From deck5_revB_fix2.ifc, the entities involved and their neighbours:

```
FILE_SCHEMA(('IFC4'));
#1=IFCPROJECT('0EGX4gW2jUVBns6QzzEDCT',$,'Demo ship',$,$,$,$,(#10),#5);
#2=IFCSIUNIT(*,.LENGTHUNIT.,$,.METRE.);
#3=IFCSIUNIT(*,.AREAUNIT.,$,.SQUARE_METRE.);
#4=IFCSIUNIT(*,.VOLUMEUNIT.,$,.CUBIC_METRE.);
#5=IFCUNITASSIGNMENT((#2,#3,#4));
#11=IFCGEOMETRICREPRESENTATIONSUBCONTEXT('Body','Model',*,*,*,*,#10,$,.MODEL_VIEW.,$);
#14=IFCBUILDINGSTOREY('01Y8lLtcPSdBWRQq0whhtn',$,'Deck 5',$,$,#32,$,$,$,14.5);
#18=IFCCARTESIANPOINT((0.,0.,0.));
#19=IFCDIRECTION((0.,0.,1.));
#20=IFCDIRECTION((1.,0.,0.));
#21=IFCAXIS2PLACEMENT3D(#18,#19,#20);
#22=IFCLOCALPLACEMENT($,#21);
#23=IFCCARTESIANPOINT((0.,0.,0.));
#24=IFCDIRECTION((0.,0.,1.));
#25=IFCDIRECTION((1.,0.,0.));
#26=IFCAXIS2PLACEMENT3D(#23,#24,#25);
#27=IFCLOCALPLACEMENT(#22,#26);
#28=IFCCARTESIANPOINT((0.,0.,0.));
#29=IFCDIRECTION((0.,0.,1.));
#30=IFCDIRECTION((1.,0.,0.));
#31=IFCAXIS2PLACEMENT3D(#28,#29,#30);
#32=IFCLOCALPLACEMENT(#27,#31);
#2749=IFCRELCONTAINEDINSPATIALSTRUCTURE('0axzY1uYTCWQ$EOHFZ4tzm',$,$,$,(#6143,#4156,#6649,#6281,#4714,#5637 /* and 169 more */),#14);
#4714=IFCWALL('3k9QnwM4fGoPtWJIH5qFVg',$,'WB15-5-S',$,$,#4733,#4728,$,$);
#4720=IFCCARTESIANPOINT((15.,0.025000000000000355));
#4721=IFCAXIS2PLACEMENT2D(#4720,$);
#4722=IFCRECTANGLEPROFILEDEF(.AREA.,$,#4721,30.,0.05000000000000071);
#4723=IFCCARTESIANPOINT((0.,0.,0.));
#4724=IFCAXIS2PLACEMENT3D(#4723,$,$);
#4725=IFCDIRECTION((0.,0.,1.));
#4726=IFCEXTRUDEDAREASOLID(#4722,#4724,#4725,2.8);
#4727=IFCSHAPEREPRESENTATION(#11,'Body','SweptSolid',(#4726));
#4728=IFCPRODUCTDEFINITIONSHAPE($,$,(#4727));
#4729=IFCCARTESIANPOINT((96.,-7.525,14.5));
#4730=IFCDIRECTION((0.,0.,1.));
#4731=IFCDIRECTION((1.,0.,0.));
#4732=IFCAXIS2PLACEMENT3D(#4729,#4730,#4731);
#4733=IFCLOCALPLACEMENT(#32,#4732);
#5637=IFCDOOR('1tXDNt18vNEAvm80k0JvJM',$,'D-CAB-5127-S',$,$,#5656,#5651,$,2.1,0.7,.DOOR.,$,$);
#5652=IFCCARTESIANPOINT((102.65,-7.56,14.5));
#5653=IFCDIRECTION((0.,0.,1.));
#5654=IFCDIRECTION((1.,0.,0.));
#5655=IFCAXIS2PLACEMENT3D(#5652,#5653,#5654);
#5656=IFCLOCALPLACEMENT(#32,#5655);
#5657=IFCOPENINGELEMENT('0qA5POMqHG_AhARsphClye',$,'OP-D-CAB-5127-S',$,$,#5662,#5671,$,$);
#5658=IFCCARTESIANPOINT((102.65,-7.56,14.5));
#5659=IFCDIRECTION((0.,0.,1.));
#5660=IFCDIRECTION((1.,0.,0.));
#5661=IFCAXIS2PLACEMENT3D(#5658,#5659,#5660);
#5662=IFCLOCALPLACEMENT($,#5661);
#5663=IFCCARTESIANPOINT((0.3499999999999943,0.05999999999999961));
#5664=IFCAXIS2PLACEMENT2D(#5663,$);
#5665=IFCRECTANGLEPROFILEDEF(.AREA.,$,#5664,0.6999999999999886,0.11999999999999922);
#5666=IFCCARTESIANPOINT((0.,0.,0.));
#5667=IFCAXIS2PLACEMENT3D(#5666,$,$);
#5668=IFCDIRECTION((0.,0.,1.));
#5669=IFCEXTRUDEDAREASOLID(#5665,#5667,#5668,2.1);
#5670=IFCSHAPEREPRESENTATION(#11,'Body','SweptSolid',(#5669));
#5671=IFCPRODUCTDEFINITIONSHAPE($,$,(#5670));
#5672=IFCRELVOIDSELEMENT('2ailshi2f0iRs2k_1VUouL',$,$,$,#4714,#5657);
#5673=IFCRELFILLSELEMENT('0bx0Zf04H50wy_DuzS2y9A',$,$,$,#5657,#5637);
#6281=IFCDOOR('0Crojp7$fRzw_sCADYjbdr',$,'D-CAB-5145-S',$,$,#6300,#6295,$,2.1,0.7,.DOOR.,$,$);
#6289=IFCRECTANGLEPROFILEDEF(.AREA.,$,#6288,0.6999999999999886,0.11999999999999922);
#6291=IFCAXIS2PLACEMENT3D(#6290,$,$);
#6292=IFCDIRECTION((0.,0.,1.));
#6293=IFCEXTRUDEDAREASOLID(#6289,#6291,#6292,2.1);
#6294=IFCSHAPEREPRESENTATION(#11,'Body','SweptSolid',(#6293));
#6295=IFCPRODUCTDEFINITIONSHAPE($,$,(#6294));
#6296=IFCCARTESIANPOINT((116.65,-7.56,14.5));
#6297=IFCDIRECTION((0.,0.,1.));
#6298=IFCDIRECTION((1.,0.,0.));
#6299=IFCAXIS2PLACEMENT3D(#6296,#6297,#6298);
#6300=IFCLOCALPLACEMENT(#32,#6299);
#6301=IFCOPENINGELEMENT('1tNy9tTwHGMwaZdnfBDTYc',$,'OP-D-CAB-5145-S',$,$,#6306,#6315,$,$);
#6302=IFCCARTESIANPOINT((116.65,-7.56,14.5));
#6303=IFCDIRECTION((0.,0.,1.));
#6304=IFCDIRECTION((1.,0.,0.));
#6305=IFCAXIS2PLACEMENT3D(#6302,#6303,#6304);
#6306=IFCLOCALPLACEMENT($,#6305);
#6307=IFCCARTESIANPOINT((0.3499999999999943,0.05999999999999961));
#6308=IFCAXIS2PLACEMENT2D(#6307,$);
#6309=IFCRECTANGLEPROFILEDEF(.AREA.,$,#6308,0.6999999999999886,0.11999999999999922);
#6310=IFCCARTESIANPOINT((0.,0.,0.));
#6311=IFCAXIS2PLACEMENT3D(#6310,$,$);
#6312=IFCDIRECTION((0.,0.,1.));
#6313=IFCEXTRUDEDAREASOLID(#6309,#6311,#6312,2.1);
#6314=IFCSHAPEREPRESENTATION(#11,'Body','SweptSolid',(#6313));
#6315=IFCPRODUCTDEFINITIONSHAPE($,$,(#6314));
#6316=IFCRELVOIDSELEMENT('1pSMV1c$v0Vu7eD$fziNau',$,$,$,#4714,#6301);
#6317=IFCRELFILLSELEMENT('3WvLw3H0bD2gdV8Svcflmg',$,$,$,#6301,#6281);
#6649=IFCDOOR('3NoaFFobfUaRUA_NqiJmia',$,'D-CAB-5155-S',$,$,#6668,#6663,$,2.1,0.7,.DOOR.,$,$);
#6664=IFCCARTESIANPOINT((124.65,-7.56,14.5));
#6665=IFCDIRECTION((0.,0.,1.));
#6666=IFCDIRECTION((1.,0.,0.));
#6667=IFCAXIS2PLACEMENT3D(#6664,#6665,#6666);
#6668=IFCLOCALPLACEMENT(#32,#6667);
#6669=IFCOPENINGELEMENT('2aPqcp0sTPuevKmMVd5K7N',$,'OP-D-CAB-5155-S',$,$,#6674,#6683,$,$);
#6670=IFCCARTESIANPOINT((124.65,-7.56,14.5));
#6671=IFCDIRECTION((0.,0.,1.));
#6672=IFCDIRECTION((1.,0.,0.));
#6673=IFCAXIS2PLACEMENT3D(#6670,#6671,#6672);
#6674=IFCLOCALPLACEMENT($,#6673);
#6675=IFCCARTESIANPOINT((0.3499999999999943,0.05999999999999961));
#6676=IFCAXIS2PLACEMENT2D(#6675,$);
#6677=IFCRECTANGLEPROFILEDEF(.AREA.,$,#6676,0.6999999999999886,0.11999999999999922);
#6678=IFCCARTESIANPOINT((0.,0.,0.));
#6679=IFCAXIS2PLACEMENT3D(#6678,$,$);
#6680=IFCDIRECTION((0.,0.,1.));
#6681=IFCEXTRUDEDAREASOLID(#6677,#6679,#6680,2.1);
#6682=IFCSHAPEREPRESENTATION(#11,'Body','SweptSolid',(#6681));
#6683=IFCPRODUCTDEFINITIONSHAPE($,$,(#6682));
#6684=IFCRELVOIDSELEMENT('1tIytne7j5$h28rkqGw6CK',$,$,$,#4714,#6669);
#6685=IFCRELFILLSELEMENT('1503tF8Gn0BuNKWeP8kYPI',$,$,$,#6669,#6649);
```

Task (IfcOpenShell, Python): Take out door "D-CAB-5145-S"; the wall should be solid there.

```python
import ifcopenshell
import ifcopenshell.api.feature
import ifcopenshell.api.root
import ifcopenshell.geom
import ifcopenshell.util.shape

model = ifcopenshell.open("deck5_revB_fix2.ifc")
settings = ifcopenshell.geom.settings()


def volume(element):
    """Net volume in cubic metres, openings subtracted."""
    shape = ifcopenshell.geom.create_shape(settings, element)
    return ifcopenshell.util.shape.get_volume(shape.geometry)


door = model.by_guid("0Crojp7$fRzw_sCADYjbdr")
opening = door.FillsVoids[0].RelatingOpeningElement
wall = opening.VoidsElements[0].RelatingBuildingElement
before = volume(wall)

ifcopenshell.api.root.remove_product(model, product=door)
ifcopenshell.api.feature.remove_feature(model, feature=opening)

after = volume(wall)

print(f"wall volume {before:.3f} -> {after:.3f} m3")

model.write("deck5_revB_fix2-out.ifc")
```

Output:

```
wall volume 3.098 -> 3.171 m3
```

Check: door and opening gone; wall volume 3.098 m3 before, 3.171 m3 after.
